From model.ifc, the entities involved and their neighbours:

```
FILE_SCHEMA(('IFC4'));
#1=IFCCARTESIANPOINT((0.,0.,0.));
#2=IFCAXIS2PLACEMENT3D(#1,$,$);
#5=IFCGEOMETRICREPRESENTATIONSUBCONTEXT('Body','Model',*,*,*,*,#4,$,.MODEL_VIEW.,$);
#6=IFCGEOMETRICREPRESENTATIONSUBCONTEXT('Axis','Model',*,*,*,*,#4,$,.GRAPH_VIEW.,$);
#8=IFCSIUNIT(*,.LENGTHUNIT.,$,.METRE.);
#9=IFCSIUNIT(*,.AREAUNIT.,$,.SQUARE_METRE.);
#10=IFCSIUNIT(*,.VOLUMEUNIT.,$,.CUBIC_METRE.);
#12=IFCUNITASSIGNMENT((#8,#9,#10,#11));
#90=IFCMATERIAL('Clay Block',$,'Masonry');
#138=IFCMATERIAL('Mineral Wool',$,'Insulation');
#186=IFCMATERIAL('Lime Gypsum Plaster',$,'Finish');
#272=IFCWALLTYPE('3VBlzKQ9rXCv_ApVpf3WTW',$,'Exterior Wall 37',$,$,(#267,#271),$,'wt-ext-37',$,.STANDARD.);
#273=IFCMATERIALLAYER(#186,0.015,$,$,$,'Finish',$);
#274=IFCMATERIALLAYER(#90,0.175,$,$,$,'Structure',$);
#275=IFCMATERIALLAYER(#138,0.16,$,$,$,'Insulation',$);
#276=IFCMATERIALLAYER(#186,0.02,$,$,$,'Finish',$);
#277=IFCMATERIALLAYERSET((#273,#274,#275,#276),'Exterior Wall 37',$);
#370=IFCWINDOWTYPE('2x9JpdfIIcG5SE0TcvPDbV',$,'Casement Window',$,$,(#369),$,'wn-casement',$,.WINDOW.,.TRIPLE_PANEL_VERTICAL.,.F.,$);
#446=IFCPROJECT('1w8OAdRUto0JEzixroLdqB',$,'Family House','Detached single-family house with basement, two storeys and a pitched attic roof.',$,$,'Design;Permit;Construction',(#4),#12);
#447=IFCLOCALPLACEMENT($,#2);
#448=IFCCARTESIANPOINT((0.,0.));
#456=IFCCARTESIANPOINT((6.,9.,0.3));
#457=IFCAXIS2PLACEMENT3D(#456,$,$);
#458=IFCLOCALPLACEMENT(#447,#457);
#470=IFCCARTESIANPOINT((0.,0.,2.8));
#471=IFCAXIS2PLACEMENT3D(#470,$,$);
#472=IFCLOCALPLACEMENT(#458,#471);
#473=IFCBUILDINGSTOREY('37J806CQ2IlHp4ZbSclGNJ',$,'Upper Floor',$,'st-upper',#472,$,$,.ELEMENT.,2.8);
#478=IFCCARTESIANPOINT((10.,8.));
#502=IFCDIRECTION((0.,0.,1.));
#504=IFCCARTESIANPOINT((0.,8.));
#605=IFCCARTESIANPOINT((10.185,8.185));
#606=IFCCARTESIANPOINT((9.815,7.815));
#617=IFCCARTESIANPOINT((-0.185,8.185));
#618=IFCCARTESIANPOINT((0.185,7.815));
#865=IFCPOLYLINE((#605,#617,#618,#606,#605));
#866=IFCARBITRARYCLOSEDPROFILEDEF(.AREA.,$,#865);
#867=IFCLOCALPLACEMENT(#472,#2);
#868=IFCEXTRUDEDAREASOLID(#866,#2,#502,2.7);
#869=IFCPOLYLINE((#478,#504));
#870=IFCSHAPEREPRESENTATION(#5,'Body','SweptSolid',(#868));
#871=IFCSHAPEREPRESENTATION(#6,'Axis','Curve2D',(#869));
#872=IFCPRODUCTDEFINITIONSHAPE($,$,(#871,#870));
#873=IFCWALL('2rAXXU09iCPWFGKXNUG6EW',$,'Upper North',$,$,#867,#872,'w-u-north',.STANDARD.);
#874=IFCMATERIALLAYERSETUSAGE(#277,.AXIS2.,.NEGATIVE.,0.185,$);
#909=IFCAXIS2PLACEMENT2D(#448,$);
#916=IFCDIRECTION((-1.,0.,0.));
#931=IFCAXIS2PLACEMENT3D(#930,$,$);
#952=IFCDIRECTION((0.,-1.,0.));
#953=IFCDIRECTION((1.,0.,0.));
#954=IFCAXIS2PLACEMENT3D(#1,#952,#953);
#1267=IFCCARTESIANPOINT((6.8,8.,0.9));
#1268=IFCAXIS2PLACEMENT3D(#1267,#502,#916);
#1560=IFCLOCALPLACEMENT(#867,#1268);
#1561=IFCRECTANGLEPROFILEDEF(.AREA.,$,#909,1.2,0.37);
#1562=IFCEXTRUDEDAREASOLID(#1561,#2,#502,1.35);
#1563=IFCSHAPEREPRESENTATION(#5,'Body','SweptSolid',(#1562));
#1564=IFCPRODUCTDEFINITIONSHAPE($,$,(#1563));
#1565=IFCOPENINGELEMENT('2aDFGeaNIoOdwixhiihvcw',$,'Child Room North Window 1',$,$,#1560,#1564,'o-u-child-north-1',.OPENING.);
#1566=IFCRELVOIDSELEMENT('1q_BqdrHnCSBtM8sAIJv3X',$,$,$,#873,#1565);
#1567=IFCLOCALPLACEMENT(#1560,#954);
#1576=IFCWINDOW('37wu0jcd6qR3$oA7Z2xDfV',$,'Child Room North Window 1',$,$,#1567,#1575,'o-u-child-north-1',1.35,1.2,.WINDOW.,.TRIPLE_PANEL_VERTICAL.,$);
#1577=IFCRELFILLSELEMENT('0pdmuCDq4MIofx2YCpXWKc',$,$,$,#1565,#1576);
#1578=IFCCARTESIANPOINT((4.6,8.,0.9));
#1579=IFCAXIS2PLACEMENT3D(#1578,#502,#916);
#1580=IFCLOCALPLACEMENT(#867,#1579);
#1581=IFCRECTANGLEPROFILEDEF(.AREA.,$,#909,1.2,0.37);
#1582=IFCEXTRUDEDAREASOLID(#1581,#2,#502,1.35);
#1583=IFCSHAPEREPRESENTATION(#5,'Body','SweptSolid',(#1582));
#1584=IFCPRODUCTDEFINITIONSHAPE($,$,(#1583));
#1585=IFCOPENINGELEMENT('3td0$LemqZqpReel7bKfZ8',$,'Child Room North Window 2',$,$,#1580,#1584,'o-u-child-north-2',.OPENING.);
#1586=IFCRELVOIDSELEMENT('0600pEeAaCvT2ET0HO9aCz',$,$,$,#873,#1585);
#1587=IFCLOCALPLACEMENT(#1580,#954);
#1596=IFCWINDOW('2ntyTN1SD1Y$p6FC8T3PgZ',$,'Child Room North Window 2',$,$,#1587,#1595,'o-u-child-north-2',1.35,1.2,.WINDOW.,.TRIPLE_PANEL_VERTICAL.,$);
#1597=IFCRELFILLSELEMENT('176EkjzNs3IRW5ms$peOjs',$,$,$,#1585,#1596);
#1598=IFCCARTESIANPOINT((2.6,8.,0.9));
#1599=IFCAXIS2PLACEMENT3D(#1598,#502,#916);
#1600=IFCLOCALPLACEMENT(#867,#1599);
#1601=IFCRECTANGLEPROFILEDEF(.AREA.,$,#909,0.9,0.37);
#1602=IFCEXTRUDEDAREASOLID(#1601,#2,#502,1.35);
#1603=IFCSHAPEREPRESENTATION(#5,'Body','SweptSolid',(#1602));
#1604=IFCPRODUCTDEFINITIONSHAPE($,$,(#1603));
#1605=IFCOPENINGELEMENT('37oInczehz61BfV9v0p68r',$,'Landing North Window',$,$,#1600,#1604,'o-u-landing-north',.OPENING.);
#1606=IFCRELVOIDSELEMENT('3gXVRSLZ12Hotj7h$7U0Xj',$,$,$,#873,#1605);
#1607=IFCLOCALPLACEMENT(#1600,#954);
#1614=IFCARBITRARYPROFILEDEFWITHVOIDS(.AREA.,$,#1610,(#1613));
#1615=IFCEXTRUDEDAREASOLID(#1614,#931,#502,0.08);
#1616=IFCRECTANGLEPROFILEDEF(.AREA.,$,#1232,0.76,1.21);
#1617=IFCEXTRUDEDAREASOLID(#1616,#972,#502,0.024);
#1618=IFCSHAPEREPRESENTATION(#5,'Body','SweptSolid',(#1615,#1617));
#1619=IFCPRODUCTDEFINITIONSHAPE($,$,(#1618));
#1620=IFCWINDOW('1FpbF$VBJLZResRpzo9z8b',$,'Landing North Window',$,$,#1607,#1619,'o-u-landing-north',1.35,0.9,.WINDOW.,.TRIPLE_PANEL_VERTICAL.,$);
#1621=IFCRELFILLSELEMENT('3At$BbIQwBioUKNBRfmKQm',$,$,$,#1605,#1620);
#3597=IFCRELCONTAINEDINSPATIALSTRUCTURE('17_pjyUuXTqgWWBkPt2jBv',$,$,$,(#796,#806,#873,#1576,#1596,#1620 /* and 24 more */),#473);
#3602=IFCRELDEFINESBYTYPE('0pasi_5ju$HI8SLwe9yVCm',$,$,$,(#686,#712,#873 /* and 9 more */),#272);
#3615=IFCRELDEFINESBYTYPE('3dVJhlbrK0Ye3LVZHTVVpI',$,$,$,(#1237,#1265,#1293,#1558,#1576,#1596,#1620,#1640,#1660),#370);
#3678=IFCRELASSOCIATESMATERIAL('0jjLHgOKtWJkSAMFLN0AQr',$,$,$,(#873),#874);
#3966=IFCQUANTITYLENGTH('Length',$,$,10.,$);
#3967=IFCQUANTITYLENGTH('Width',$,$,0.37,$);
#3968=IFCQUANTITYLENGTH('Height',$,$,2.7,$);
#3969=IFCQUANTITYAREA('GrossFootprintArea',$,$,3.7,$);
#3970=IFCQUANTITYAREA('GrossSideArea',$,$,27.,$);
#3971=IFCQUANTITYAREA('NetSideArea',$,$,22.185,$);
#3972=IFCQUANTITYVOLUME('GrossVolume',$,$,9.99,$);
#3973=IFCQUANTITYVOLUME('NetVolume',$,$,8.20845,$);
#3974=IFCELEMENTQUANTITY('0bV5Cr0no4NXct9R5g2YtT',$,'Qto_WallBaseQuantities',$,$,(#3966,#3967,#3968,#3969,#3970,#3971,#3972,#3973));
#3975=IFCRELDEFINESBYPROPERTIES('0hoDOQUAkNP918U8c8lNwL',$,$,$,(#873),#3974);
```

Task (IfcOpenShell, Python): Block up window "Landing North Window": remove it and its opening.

```python
import ifcopenshell
import ifcopenshell.api.feature
import ifcopenshell.api.pset
import ifcopenshell.api.root
import ifcopenshell.geom
import ifcopenshell.util.element
import ifcopenshell.util.shape
import ifcopenshell.util.unit

model = ifcopenshell.open("model.ifc")
area_scale = ifcopenshell.util.unit.calculate_unit_scale(model, "AREAUNIT")
volume_scale = ifcopenshell.util.unit.calculate_unit_scale(model, "VOLUMEUNIT")
settings = ifcopenshell.geom.settings()


def volume(element):
    """Net volume in cubic metres, openings subtracted."""
    shape = ifcopenshell.geom.create_shape(settings, element)
    return ifcopenshell.util.shape.get_volume(shape.geometry)


window = model.by_guid("1FpbF$VBJLZResRpzo9z8b")
opening = window.FillsVoids[0].RelatingOpeningElement
wall = opening.VoidsElements[0].RelatingBuildingElement
before = volume(wall)

ifcopenshell.api.root.remove_product(model, product=window)
ifcopenshell.api.feature.remove_feature(model, feature=opening)

after = volume(wall)
thickness = 0.37  # wall thickness in metres

# Update the wall's stored quantities.
qto = model.by_id(ifcopenshell.util.element.get_pset(wall, "Qto_WallBaseQuantities", should_inherit=False)["id"])
ifcopenshell.api.pset.edit_qto(model, qto=qto, properties={
    "NetSideArea": after / thickness / area_scale,
    "NetVolume": after / volume_scale,
})

print(f"wall volume {before:.3f} -> {after:.3f} m3")

model.write("model-out.ifc")
```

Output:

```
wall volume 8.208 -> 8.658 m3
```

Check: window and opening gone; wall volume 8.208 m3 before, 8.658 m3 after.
